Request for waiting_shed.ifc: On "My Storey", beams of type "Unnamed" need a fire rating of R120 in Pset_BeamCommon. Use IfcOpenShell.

First a look at what the model holds.

```python
import ifcopenshell
import ifcopenshell.util.element

model = ifcopenshell.open("waiting_shed.ifc")
print(model.schema)
storey = next(s for s in model.by_type("IfcBuildingStorey") if s.Name == "My Storey")
beams = [e for e in ifcopenshell.util.element.get_decomposition(storey) if e.is_a("IfcBeam")]
seen = {}
for e in beams:
    element_type = ifcopenshell.util.element.get_type(e)
    key = (element_type.Name if element_type != e and element_type else None, ifcopenshell.util.element.get_pset(e, "Pset_BeamCommon", "FireRating"))
    seen[key] = seen.get(key, 0) + 1
for (name, value), count in sorted(seen.items(), key=str):
    print(count, "x", name, "|", value)
```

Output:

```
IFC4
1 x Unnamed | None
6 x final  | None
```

```python
import ifcopenshell
import ifcopenshell.api.pset
import ifcopenshell.util.element

model = ifcopenshell.open("waiting_shed.ifc")

storey = next(s for s in model.by_type("IfcBuildingStorey") if s.Name == "My Storey")
beams = [e for e in ifcopenshell.util.element.get_decomposition(storey) if e.is_a("IfcBeam")]

count = 0
for e in beams:
    element_type = ifcopenshell.util.element.get_type(e)
    if element_type in (None, e) or element_type.Name != "Unnamed":
        continue
    # add_pset returns the element's existing set when there is one.
    pset = ifcopenshell.api.pset.add_pset(model, product=e, name="Pset_BeamCommon")
    ifcopenshell.api.pset.edit_pset(model, pset=pset, properties={"FireRating": "R120"})
    count += 1

print(count, "beams updated")

model.write("waiting_shed-out.ifc")
```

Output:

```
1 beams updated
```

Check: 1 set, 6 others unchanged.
